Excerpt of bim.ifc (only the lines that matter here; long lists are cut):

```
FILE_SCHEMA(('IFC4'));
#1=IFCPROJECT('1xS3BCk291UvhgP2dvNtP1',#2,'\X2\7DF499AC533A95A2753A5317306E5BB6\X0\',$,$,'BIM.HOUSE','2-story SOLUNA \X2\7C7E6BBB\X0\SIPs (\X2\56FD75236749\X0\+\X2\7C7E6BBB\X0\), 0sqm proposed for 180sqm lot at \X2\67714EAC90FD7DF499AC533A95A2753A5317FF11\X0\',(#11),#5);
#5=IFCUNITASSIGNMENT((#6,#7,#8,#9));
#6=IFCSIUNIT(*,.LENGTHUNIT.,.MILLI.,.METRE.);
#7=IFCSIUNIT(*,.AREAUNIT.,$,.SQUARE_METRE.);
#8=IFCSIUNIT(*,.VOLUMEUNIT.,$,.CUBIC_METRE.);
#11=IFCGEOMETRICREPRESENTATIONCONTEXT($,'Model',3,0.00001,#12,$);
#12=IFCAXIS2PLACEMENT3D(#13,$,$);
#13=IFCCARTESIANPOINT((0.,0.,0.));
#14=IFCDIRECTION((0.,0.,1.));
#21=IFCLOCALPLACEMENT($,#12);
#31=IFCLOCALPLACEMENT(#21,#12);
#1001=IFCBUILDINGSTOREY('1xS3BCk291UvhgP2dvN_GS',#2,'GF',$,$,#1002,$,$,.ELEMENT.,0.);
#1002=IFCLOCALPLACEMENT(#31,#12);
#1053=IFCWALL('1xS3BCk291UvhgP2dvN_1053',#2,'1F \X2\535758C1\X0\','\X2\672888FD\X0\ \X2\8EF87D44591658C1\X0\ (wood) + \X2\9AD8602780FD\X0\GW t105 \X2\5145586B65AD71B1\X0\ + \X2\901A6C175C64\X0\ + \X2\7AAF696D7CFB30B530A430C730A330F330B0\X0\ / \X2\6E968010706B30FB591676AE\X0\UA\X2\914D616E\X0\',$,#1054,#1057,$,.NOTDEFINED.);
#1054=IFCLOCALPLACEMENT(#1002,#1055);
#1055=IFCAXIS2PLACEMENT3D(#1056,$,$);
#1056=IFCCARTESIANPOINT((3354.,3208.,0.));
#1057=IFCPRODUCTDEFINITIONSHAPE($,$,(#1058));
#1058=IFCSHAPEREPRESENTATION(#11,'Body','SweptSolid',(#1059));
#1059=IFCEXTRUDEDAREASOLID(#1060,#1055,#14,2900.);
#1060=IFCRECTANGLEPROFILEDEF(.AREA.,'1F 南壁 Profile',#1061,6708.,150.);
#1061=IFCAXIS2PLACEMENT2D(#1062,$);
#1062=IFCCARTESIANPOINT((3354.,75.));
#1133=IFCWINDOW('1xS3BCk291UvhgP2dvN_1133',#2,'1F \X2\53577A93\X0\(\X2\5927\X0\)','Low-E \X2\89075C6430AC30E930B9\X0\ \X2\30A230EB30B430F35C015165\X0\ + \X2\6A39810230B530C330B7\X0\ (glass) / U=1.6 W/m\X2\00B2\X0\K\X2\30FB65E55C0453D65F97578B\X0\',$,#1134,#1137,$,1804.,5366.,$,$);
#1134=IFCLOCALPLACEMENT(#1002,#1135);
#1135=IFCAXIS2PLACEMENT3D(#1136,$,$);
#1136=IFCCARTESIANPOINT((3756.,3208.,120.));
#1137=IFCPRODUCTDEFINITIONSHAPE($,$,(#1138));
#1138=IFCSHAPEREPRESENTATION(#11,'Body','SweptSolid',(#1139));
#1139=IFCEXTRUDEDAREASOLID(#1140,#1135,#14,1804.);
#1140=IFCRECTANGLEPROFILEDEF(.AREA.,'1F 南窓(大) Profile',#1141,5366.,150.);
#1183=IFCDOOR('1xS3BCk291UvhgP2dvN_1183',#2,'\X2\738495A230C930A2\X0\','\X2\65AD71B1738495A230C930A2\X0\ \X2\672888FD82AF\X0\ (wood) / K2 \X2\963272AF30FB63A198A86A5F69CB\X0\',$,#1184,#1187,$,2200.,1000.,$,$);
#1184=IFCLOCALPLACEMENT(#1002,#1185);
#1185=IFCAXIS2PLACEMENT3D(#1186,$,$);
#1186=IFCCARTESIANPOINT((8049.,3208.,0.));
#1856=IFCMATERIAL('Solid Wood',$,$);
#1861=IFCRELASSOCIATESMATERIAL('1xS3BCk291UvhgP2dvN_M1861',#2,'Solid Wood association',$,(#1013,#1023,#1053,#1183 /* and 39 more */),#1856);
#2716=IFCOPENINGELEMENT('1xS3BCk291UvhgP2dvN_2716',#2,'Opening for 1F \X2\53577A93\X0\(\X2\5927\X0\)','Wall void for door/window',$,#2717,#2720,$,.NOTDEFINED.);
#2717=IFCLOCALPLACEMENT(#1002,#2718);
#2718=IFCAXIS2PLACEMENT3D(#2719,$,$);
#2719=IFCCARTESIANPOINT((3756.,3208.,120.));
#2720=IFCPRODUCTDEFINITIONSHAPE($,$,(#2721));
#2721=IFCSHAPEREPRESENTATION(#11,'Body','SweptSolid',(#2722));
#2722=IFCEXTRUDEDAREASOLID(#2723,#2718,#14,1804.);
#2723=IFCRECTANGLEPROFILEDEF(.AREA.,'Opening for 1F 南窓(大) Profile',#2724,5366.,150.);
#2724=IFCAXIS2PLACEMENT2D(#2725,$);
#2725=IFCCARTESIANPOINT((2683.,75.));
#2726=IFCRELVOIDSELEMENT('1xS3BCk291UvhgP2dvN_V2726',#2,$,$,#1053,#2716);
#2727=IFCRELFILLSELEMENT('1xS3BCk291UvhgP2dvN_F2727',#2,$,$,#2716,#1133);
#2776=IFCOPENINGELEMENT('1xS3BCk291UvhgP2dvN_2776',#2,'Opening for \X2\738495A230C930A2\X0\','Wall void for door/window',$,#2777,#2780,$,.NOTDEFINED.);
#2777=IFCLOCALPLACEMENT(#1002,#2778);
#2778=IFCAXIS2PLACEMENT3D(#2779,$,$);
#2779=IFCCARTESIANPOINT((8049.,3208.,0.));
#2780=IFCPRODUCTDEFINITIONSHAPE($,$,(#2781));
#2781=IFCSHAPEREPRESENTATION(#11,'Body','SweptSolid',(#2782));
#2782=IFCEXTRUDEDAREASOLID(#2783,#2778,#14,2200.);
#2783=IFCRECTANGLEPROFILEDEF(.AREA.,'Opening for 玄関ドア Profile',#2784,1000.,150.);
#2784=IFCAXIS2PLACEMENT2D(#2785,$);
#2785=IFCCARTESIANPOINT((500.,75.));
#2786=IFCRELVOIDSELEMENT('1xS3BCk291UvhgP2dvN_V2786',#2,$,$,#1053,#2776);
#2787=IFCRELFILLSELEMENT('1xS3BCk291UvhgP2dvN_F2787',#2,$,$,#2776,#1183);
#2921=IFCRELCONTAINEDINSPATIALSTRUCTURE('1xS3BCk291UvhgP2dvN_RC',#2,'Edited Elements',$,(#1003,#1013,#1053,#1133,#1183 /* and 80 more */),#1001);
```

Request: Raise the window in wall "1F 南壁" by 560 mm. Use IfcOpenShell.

```python
import numpy as np
import ifcopenshell
import ifcopenshell.api.geometry
import ifcopenshell.util.placement
import ifcopenshell.util.unit

model = ifcopenshell.open("bim.ifc")
unit_scale = ifcopenshell.util.unit.calculate_unit_scale(model)

window = model.by_guid("1xS3BCk291UvhgP2dvN_1133")
opening = window.FillsVoids[0].RelatingOpeningElement
dz = 560.0

shift = np.array([0.0, 0.0, dz])
# The window is not placed relative to its opening, so move both.
for product in (opening, window):
    matrix = ifcopenshell.util.placement.get_local_placement(product.ObjectPlacement)
    matrix[:3, 3] += shift
    ifcopenshell.api.geometry.edit_object_placement(model, product=product, matrix=matrix, is_si=False)

print(f"moved by {dz * unit_scale:+.3f} m")

model.write("bim_edited.ifc")
```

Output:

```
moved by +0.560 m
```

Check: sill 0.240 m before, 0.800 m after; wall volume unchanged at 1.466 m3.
